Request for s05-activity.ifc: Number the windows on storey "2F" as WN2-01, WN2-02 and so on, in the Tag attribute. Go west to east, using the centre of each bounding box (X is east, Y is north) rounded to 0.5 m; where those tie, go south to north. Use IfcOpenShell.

First a look at what the model holds.

```python
import ifcopenshell
import ifcopenshell.util.element
import ifcopenshell.util.placement

model = ifcopenshell.open("s05-activity.ifc")
print(model.schema)
storey = next(s for s in model.by_type("IfcBuildingStorey") if s.Name == "2F")
windows = [e for e in ifcopenshell.util.element.get_decomposition(storey) if e.is_a("IfcWindow")]
for e in sorted(windows, key=lambda e: e.id()):
    origin = ifcopenshell.util.placement.get_local_placement(e.ObjectPlacement)[:3, 3]
    print(e.id(), e.Tag, e.Name, origin.round(2) + 0.0, sep=" | ")
```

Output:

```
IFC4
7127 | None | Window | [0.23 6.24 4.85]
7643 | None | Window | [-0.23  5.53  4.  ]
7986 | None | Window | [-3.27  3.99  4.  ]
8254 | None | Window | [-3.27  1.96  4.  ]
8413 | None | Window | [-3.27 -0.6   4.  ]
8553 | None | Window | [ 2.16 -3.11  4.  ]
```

```python
import ifcopenshell
import ifcopenshell.geom
import ifcopenshell.util.element
import ifcopenshell.util.shape

model = ifcopenshell.open("s05-activity.ifc")
settings = ifcopenshell.geom.settings()
settings.set("use-world-coords", True)


def centre(element):
    shape = ifcopenshell.geom.create_shape(settings, element)
    return ifcopenshell.util.shape.get_bbox_centroid(shape.geometry)


storey = next(s for s in model.by_type("IfcBuildingStorey") if s.Name == "2F")
windows = [e for e in ifcopenshell.util.element.get_decomposition(storey) if e.is_a("IfcWindow")]

# Insertion points can sit at a corner or the storey origin, so sort by the geometry (in metres).
centres = {e: centre(e) for e in windows}
windows.sort(key=lambda e: (round(centres[e][0] / 0.5), centres[e][1]))

for i, e in enumerate(windows, start=1):
    number = f"WN2-{i:02d}"
    e.Tag = number
    print(e.id(), number)

model.write("s05-activity_edited.ifc")
```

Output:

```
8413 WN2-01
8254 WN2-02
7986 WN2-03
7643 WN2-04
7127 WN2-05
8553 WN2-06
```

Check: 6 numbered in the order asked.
